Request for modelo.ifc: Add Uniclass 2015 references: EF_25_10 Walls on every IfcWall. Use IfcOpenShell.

First a look at what the model holds.

```python
import ifcopenshell

model = ifcopenshell.open("modelo.ifc")
print(model.schema)
print("classifications:", [c.Name for c in model.by_type("IfcClassification")])
for ifc_class in ("IfcDoor", "IfcRoof", "IfcStair", "IfcWall", "IfcWindow"):
    print(ifc_class, len(model.by_type(ifc_class)))
```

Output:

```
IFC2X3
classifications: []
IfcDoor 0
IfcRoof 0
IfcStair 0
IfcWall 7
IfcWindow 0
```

```python
import ifcopenshell
import ifcopenshell.api.classification

model = ifcopenshell.open("modelo.ifc")

# IFC2X3 requires Source and Edition and has no link from the project to the system.
system = model.create_entity("IfcClassification", Source="NBS", Edition="2015", Name="Uniclass 2015")

codes = {
    "IfcWall": ("EF_25_10", "Walls"),
}
for ifc_class, (code, name) in codes.items():
    products = model.by_type(ifc_class)
    ifcopenshell.api.classification.add_reference(
        model, products=products, classification=system, identification=code, name=name
    )
    print(code, len(products))

model.write("modelo_edited.ifc")
```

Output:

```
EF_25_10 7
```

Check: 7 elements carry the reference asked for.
